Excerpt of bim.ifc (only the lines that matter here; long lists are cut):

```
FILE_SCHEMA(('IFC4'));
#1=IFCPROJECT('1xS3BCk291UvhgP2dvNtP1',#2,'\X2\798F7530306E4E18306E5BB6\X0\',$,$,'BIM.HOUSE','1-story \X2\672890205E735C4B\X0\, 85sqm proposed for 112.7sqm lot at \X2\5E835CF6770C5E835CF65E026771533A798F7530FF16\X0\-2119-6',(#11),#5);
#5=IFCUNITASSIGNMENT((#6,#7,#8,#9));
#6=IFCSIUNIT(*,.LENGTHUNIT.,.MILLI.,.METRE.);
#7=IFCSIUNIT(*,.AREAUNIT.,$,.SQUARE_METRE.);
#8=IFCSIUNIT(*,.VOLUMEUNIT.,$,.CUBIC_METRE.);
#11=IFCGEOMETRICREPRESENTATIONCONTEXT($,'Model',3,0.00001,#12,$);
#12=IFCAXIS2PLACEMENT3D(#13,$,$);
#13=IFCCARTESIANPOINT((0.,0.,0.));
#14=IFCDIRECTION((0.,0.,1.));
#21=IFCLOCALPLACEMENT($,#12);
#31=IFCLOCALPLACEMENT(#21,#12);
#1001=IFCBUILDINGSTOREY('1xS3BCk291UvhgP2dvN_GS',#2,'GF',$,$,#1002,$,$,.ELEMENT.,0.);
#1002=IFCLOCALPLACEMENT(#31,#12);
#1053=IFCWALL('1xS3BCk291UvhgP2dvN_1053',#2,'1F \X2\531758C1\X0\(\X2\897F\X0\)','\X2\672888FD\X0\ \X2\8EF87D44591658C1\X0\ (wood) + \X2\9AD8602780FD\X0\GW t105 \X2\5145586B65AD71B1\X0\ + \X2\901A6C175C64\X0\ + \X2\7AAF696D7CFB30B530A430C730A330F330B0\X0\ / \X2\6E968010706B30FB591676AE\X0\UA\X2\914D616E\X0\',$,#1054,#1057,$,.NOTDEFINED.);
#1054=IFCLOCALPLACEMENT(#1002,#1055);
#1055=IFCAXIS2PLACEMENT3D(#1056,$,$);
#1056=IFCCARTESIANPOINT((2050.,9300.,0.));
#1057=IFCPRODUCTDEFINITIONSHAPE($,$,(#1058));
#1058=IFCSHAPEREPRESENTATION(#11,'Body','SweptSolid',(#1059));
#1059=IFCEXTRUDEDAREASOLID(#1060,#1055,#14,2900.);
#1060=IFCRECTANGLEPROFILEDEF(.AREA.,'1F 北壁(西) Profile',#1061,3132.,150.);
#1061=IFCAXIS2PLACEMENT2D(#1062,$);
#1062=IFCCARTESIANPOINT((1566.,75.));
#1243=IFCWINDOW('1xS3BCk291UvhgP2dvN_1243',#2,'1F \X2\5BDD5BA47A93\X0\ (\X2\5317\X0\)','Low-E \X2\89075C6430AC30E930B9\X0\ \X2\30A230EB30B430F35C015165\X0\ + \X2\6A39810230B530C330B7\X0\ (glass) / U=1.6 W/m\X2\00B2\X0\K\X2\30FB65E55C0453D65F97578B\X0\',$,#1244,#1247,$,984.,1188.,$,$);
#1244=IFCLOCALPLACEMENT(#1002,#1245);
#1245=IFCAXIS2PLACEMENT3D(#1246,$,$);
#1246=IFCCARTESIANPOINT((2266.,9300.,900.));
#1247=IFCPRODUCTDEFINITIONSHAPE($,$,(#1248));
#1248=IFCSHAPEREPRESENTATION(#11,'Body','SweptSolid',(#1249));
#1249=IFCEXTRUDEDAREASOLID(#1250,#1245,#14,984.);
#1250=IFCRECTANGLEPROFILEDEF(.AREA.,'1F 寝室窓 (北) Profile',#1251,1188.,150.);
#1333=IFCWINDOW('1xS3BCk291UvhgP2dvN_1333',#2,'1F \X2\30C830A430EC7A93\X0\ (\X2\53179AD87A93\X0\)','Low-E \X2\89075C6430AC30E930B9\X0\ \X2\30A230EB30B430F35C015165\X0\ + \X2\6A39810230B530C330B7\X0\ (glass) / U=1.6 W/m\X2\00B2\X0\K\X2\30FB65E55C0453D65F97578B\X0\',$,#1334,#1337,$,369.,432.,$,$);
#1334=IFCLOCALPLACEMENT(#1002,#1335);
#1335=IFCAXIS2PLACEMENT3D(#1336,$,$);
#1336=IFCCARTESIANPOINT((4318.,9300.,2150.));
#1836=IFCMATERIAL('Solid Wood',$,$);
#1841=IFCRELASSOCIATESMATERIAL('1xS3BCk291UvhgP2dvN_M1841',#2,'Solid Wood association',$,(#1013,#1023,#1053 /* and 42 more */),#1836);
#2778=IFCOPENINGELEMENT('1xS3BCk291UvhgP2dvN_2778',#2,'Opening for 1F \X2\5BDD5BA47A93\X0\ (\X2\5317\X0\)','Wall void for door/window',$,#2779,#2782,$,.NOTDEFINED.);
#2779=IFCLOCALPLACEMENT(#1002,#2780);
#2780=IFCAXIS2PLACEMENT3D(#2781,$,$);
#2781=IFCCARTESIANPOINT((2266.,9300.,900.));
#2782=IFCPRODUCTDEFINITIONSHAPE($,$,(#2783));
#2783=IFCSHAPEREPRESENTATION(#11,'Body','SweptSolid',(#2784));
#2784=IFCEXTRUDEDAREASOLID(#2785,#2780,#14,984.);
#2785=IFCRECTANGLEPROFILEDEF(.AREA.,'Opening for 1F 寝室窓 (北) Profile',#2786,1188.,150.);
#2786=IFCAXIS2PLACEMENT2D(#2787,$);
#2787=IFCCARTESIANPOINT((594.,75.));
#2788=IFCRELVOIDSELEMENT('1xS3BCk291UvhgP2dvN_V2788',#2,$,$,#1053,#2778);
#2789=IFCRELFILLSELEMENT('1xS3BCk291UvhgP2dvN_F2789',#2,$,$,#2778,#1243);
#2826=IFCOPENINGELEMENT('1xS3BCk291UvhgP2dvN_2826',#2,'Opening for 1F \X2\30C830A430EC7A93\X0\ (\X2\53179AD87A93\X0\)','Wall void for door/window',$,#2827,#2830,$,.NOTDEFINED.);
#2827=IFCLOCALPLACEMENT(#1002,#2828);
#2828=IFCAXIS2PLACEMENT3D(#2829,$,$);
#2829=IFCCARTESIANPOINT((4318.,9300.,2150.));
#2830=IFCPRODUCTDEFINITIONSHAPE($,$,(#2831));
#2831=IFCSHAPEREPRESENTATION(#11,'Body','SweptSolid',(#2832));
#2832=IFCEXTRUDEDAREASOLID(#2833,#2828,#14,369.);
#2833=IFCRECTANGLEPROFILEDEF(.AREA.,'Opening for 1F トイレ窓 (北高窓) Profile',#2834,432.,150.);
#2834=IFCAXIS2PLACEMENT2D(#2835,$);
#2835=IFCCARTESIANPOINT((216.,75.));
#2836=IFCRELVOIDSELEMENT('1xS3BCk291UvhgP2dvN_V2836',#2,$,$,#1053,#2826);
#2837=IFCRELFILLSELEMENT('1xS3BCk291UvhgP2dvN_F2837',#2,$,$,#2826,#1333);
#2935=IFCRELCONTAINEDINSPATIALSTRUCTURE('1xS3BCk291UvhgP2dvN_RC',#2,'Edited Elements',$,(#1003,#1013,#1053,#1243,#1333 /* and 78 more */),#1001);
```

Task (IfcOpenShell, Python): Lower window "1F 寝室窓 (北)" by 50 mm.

```python
import numpy as np
import ifcopenshell
import ifcopenshell.api.geometry
import ifcopenshell.util.placement
import ifcopenshell.util.unit

model = ifcopenshell.open("bim.ifc")
unit_scale = ifcopenshell.util.unit.calculate_unit_scale(model)

window = model.by_id(1243)
opening = window.FillsVoids[0].RelatingOpeningElement
dz = -50.0

shift = np.array([0.0, 0.0, dz])
# The window is not placed relative to its opening, so move both.
for product in (opening, window):
    matrix = ifcopenshell.util.placement.get_local_placement(product.ObjectPlacement)
    matrix[:3, 3] += shift
    ifcopenshell.api.geometry.edit_object_placement(model, product=product, matrix=matrix, is_si=False)

print(f"moved by {dz * unit_scale:+.3f} m")

model.write("bim_v2.ifc")
```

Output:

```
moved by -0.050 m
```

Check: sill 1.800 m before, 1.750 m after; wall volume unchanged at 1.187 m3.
